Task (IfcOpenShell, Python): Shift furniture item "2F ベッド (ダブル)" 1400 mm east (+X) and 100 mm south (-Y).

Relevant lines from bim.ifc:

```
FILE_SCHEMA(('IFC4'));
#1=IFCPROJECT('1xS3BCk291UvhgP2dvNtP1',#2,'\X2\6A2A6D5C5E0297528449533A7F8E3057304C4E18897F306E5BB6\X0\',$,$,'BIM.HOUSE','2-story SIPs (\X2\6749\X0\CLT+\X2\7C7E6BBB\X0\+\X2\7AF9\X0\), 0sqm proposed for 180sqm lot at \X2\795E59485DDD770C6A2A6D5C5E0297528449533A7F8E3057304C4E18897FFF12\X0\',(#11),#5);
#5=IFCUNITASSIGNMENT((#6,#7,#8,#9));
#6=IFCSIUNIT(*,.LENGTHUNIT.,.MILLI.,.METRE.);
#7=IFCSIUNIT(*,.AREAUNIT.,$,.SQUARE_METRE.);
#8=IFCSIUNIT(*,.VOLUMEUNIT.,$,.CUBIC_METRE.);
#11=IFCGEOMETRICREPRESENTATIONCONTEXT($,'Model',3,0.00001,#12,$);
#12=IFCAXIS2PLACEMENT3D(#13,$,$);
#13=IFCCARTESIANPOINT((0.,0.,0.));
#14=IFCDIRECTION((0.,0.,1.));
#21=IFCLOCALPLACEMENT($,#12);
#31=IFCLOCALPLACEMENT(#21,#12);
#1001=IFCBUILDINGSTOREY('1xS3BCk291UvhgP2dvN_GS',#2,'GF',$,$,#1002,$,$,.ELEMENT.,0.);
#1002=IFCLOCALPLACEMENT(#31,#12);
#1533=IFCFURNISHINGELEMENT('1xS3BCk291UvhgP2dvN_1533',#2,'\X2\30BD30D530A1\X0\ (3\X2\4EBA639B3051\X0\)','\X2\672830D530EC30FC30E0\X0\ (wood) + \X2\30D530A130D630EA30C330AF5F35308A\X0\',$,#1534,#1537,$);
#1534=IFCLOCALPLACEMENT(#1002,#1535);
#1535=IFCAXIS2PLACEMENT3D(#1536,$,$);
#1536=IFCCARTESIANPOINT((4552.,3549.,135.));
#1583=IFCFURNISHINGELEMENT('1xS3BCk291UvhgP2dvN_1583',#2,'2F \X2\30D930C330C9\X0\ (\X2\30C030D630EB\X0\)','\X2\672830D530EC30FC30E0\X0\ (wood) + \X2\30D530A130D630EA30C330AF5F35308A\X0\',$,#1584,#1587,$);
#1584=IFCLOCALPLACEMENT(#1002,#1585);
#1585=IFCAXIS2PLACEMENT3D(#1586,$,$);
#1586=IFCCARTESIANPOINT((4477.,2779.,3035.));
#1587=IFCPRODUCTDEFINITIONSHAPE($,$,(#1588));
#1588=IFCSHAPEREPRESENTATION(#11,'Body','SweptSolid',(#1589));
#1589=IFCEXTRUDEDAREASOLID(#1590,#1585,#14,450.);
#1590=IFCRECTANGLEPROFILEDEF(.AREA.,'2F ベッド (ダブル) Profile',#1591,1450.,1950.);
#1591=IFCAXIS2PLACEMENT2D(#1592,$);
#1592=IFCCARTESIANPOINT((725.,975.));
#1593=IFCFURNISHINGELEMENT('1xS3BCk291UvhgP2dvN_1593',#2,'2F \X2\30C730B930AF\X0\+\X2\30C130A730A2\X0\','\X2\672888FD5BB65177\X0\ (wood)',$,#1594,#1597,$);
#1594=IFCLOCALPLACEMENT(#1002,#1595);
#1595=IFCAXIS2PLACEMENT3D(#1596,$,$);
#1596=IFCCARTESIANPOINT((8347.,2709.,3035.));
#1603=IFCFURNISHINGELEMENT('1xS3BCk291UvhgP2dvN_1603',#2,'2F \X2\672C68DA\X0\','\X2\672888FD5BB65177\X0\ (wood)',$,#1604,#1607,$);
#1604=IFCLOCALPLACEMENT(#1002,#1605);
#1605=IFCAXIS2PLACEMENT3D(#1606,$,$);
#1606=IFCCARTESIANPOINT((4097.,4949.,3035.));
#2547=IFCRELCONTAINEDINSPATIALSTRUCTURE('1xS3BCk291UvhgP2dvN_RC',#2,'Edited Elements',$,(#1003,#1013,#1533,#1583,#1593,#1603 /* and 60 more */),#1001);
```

```python
import ifcopenshell
import ifcopenshell.api.geometry
import ifcopenshell.util.placement
import ifcopenshell.util.unit

model = ifcopenshell.open("bim.ifc")
unit_scale = ifcopenshell.util.unit.calculate_unit_scale(model)

item = model.by_id(1583)
matrix = ifcopenshell.util.placement.get_local_placement(item.ObjectPlacement)
matrix[0, 3] += 1.4 / unit_scale
matrix[1, 3] -= 0.1 / unit_scale
ifcopenshell.api.geometry.edit_object_placement(model, product=item, matrix=matrix, is_si=False)

print(ifcopenshell.util.placement.get_local_placement(item.ObjectPlacement).round(3) + 0.0)

model.write("bim_rev.ifc")
```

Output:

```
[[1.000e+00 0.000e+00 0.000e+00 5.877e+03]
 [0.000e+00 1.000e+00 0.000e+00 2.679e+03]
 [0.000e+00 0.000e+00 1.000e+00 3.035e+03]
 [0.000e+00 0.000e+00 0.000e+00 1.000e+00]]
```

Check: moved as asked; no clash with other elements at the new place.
